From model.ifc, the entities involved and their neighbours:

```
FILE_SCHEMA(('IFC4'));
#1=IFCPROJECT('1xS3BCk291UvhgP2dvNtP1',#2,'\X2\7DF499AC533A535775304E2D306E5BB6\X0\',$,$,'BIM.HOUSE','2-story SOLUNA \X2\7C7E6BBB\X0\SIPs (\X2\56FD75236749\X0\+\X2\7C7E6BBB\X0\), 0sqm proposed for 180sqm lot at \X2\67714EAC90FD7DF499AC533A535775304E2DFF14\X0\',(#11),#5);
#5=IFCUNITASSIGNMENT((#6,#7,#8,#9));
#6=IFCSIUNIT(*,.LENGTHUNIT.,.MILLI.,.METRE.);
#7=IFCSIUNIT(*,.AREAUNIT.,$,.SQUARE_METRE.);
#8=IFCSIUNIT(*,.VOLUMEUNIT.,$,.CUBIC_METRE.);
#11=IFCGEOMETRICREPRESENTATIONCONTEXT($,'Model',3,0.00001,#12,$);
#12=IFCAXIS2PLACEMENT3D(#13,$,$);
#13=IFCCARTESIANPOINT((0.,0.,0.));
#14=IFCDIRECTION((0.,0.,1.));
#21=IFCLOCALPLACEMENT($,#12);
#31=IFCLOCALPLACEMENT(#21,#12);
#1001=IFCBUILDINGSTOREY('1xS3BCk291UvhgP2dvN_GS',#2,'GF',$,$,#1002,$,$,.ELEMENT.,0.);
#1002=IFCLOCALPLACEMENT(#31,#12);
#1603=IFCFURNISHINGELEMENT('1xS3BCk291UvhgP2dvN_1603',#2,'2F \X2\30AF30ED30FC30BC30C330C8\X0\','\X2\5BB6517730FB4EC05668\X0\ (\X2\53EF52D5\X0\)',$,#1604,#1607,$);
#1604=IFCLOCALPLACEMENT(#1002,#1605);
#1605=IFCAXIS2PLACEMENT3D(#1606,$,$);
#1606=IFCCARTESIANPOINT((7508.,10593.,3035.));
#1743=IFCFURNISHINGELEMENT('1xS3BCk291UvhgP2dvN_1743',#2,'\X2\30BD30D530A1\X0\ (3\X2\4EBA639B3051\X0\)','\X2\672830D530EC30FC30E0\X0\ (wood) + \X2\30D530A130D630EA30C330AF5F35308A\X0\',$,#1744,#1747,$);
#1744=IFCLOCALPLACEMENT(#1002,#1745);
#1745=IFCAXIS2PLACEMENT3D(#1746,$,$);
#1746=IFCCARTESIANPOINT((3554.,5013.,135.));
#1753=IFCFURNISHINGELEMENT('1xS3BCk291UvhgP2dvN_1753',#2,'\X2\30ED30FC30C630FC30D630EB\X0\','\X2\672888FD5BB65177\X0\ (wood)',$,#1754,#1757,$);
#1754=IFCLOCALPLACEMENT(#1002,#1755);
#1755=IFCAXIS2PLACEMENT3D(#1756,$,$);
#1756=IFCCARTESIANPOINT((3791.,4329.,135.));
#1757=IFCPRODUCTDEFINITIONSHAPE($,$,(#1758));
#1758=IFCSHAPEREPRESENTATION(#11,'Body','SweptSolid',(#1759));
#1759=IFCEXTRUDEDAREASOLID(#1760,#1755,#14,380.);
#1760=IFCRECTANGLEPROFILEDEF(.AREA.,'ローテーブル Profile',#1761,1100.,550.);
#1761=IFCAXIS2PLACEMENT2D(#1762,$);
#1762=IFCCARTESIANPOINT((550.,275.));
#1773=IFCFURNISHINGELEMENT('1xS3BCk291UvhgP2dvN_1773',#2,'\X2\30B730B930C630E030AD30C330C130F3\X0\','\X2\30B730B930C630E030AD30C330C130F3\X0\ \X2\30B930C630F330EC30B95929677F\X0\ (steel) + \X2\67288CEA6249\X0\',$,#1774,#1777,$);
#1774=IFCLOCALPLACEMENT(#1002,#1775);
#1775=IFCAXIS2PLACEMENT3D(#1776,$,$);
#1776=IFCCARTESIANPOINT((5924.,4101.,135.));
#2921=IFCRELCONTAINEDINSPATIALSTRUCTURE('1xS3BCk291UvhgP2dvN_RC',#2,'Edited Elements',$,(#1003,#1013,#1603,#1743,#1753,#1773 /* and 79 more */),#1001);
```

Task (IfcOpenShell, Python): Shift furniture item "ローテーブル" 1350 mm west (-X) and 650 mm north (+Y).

```python
import ifcopenshell
import ifcopenshell.api.geometry
import ifcopenshell.util.placement

model = ifcopenshell.open("model.ifc")

item = model.by_guid("1xS3BCk291UvhgP2dvN_1753")
matrix = ifcopenshell.util.placement.get_local_placement(item.ObjectPlacement)
matrix[0, 3] -= 1350.0
matrix[1, 3] += 650.0
ifcopenshell.api.geometry.edit_object_placement(model, product=item, matrix=matrix, is_si=False)

print(ifcopenshell.util.placement.get_local_placement(item.ObjectPlacement).round(3) + 0.0)

model.write("model_rev.ifc")
```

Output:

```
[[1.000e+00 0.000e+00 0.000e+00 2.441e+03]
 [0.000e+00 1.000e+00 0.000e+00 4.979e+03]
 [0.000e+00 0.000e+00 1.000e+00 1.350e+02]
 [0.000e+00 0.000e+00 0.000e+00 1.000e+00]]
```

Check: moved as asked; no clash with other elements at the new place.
